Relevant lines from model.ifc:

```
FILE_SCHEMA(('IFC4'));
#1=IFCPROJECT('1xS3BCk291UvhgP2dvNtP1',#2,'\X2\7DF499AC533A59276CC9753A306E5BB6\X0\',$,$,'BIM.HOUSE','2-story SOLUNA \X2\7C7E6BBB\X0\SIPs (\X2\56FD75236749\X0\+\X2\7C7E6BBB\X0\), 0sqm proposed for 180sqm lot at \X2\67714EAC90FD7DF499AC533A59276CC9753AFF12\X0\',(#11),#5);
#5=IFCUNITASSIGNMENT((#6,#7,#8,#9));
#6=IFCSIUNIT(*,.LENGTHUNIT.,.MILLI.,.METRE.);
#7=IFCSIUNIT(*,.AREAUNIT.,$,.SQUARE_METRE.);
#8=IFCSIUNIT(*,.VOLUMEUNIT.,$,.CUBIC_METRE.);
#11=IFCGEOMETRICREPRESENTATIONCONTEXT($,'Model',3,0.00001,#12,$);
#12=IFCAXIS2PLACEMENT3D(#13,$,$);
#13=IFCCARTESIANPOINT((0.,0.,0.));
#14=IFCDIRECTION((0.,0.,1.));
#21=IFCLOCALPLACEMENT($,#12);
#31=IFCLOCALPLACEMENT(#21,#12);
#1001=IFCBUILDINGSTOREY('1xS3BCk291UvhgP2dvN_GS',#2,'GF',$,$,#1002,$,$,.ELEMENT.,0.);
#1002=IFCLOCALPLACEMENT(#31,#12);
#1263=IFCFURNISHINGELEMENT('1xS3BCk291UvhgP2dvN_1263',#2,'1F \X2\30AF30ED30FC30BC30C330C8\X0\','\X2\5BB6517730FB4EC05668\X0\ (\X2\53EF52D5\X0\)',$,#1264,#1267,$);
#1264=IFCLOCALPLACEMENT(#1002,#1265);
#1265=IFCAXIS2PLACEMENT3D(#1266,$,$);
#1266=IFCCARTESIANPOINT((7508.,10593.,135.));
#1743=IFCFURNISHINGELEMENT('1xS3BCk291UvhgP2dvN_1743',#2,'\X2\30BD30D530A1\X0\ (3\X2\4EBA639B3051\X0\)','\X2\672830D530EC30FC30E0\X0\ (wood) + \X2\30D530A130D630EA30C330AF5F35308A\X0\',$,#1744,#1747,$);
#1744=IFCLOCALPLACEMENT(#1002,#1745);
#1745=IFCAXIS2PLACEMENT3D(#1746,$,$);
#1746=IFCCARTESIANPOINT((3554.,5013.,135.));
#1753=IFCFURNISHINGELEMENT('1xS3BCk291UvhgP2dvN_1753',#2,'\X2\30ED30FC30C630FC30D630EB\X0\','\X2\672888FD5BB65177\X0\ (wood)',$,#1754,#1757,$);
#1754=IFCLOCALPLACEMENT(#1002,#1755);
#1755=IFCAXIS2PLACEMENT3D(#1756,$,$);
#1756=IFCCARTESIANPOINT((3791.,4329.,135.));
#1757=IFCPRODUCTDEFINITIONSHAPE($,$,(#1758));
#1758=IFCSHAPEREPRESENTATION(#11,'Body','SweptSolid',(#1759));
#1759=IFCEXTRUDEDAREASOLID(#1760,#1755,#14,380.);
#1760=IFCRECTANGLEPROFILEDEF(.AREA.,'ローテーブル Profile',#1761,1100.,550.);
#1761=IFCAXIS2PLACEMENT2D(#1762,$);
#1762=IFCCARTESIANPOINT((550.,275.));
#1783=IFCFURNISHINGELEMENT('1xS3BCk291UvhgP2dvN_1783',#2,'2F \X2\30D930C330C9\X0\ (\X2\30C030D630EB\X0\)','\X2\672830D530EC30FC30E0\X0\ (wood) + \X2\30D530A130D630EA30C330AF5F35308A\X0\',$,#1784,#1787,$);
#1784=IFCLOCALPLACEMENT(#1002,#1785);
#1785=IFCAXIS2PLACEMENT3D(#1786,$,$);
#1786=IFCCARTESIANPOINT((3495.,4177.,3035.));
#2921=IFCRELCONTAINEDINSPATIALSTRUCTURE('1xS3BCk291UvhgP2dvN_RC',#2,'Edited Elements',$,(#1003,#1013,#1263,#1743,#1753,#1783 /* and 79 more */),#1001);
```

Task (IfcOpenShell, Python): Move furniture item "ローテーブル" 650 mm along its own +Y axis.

```python
import ifcopenshell
import ifcopenshell.api.geometry
import ifcopenshell.util.placement

model = ifcopenshell.open("model.ifc")

item = model.by_guid("1xS3BCk291UvhgP2dvN_1753")
matrix = ifcopenshell.util.placement.get_local_placement(item.ObjectPlacement)
matrix[:3, 3] += matrix[:3, 1] * 650.0
ifcopenshell.api.geometry.edit_object_placement(model, product=item, matrix=matrix, is_si=False)

print(ifcopenshell.util.placement.get_local_placement(item.ObjectPlacement).round(3) + 0.0)

model.write("model_rev.ifc")
```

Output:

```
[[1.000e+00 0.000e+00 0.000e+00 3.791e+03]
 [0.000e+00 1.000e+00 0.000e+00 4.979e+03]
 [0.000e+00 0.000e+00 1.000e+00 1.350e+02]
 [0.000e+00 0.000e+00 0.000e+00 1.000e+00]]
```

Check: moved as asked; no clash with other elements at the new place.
